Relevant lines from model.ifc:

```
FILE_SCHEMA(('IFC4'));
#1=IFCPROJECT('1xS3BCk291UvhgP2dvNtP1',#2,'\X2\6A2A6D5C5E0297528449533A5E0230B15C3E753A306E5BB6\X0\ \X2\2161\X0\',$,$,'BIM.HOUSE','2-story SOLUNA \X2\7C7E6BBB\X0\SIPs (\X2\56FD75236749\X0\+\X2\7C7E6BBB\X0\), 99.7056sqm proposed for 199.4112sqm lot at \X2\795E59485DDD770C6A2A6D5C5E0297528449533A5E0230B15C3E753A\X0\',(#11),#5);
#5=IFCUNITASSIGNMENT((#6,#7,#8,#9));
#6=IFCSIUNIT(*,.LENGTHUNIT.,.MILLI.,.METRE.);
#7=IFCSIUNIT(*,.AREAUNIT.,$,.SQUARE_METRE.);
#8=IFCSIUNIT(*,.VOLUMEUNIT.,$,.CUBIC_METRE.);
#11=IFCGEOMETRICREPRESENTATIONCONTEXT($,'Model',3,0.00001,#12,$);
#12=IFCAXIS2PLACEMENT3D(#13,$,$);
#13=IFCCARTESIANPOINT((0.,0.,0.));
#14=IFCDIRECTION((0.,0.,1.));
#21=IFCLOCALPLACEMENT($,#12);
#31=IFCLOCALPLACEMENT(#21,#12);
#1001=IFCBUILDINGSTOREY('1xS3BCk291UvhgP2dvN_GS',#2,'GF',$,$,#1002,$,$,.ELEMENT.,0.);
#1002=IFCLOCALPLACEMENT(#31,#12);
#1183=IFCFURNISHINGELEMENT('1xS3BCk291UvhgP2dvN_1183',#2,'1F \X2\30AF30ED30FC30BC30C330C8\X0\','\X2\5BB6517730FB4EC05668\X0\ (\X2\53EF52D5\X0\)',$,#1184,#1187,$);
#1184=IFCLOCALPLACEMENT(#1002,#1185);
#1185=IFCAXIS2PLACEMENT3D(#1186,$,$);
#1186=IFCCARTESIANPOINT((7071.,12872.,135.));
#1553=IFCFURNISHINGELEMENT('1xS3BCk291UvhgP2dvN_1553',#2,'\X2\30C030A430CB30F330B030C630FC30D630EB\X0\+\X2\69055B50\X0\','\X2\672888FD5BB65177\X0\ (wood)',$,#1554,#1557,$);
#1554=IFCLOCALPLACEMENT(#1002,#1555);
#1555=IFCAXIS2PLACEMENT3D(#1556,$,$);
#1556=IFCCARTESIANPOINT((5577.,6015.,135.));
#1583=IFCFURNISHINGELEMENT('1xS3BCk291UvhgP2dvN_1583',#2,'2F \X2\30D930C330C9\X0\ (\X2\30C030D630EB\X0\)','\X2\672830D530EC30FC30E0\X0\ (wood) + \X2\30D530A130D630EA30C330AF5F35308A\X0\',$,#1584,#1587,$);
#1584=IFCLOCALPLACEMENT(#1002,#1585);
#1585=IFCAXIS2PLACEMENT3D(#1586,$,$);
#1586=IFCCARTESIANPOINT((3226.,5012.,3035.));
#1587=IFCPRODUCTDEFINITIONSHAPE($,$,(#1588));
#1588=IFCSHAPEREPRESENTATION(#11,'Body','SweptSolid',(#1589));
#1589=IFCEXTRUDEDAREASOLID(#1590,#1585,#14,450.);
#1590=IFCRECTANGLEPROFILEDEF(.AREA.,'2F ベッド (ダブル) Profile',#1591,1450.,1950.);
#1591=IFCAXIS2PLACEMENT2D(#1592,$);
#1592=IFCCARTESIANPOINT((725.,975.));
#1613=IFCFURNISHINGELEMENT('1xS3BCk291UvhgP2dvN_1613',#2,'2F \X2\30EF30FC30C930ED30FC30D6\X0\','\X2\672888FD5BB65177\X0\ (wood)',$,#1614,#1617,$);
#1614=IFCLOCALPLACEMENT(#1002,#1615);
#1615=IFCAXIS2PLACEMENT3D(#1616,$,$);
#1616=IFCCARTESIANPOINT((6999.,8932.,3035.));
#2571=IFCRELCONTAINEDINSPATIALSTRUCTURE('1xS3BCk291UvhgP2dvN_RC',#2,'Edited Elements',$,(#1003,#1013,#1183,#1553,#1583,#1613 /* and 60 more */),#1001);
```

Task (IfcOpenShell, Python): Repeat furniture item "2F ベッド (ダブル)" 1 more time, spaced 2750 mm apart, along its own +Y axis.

```python
import ifcopenshell
import ifcopenshell.api.geometry
import ifcopenshell.api.root
import ifcopenshell.util.element
import ifcopenshell.util.placement

model = ifcopenshell.open("model.ifc")


def reuse_history(source, copy):
    """copy_class also copies each property set's owner history, people and application; keep the originals."""
    for rel in copy.IsDefinedBy:
        if rel.is_a("IfcRelDefinesByProperties") and (history := rel.RelatingPropertyDefinition.OwnerHistory):
            rel.RelatingPropertyDefinition.OwnerHistory = source.OwnerHistory
            ifcopenshell.util.element.remove_deep2(model, history)


source = model.by_guid("1xS3BCk291UvhgP2dvN_1583")
base = ifcopenshell.util.placement.get_local_placement(source.ObjectPlacement)
step = base[:3, 1] * 2750.0

for i in range(1, 2):
    copy = ifcopenshell.api.root.copy_class(model, product=source)
    copy.Representation = ifcopenshell.util.element.copy_deep(
        model, source.Representation, exclude=["IfcGeometricRepresentationContext", "IfcRepresentationMap"]
    )
    reuse_history(source, copy)
    matrix = base.copy()
    matrix[:3, 3] += i * step
    print("added at", matrix[:3, 3].round(3) + 0.0)
    ifcopenshell.api.geometry.edit_object_placement(model, product=copy, matrix=matrix, is_si=False)

model.write("model_v2.ifc")
```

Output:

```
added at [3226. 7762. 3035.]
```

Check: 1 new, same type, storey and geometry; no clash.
